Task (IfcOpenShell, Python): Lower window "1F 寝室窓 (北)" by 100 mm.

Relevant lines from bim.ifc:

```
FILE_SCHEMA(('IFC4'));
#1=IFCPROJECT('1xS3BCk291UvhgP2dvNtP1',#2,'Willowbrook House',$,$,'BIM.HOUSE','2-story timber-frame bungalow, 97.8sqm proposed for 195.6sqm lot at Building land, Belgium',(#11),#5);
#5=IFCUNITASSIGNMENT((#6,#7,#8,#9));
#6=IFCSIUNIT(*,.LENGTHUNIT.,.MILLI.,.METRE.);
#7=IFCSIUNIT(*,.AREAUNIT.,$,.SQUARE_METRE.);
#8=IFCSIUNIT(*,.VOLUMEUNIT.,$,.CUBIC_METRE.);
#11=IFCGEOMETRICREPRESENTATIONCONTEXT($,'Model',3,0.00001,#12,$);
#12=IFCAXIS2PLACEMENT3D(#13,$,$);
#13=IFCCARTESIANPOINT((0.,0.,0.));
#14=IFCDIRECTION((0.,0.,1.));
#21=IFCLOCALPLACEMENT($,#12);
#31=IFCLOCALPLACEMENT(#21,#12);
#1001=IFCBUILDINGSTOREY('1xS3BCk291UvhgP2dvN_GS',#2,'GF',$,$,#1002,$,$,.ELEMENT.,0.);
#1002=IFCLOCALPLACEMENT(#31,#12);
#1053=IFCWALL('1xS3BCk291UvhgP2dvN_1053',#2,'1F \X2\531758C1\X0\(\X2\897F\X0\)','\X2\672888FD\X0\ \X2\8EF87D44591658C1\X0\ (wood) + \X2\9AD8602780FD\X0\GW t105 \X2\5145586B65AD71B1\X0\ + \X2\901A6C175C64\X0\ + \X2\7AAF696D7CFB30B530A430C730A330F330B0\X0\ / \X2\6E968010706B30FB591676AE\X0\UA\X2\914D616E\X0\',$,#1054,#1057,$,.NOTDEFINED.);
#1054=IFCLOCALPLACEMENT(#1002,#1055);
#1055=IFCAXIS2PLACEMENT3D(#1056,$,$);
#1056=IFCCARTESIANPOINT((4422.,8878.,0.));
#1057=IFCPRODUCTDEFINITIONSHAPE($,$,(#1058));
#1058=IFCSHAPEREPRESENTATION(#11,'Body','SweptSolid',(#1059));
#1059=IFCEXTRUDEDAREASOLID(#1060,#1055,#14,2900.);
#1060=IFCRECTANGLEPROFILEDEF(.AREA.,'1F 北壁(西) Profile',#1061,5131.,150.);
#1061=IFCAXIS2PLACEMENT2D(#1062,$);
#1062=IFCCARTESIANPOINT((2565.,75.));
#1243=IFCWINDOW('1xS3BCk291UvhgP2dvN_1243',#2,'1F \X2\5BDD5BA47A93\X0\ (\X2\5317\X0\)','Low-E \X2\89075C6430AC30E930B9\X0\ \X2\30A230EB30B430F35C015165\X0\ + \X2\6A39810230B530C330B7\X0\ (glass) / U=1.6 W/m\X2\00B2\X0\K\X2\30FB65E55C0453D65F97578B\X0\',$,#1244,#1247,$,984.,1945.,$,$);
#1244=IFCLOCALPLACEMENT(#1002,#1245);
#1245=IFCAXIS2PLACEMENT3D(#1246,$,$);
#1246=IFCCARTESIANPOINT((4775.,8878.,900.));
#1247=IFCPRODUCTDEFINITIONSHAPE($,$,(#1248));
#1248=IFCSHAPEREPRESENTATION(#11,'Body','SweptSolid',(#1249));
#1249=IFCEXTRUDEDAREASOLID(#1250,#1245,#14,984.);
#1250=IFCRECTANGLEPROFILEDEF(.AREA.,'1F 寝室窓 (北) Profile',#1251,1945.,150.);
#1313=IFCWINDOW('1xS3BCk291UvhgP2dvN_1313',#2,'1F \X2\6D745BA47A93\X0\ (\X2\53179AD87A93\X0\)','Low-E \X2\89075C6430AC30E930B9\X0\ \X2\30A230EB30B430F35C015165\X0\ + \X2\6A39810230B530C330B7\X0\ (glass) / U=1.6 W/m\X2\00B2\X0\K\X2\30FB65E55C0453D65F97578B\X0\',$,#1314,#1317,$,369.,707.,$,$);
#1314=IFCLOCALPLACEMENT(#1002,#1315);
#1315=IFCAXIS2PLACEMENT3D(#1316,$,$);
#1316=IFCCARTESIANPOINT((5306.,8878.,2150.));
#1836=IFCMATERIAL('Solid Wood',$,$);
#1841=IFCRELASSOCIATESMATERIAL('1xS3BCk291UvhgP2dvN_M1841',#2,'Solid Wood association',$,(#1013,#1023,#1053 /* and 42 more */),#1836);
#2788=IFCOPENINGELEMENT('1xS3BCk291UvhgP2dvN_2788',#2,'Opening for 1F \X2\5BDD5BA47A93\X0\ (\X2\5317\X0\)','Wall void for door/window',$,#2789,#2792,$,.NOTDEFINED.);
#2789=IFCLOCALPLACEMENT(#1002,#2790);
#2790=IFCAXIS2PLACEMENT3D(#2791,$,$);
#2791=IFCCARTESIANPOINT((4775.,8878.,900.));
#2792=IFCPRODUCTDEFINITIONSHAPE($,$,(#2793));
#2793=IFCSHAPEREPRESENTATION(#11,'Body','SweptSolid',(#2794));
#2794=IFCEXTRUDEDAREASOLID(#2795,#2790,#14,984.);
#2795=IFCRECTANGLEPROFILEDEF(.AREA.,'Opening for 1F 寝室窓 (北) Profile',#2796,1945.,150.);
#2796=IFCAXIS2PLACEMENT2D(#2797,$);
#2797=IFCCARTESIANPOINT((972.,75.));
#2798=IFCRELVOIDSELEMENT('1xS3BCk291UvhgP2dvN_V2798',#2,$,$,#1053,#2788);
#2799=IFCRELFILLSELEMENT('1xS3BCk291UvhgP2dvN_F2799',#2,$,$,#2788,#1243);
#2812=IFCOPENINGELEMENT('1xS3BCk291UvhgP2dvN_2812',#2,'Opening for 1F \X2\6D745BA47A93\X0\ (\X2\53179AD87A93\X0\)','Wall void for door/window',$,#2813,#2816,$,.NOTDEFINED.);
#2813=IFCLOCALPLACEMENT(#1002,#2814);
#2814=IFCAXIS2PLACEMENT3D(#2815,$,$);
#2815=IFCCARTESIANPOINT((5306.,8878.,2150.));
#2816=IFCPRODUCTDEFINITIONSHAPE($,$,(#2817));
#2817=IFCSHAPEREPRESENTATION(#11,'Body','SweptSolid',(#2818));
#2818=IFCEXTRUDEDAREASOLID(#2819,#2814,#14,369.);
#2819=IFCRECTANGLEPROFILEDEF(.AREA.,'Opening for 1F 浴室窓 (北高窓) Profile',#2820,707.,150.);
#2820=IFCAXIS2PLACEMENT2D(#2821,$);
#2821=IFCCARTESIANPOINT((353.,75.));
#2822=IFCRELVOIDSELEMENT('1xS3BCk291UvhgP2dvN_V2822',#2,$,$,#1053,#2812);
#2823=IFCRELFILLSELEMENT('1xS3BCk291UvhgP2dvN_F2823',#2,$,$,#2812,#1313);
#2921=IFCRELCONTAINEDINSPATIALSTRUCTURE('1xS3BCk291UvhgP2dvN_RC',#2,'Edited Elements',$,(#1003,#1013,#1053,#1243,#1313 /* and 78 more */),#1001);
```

```python
import numpy as np
import ifcopenshell
import ifcopenshell.api.geometry
import ifcopenshell.util.placement
import ifcopenshell.util.unit

model = ifcopenshell.open("bim.ifc")
unit_scale = ifcopenshell.util.unit.calculate_unit_scale(model)

window = model.by_guid("1xS3BCk291UvhgP2dvN_1243")
opening = window.FillsVoids[0].RelatingOpeningElement
dz = -100.0

shift = np.array([0.0, 0.0, dz])
# The window is not placed relative to its opening, so move both.
for product in (opening, window):
    matrix = ifcopenshell.util.placement.get_local_placement(product.ObjectPlacement)
    matrix[:3, 3] += shift
    ifcopenshell.api.geometry.edit_object_placement(model, product=product, matrix=matrix, is_si=False)

print(f"moved by {dz * unit_scale:+.3f} m")

model.write("bim-out.ifc")
```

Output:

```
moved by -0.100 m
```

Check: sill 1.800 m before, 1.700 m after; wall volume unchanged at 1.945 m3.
